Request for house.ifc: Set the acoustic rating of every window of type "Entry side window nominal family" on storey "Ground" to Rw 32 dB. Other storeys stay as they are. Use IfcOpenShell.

First a look at what the model holds.

```python
import ifcopenshell
import ifcopenshell.util.element

model = ifcopenshell.open("house.ifc")
print(model.schema)
storey = next(s for s in model.by_type("IfcBuildingStorey") if s.Name == "Ground")
windows = [e for e in ifcopenshell.util.element.get_decomposition(storey) if e.is_a("IfcWindow")]
seen = {}
for e in windows:
    element_type = ifcopenshell.util.element.get_type(e)
    key = (element_type.Name if element_type != e and element_type else None, ifcopenshell.util.element.get_pset(e, "Pset_WindowCommon", "AcousticRating"))
    seen[key] = seen.get(key, 0) + 1
for (name, value), count in sorted(seen.items(), key=str):
    print(count, "x", name, "|", value)
```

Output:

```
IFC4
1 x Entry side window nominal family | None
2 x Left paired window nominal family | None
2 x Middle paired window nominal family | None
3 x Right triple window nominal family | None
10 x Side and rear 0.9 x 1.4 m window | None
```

```python
import ifcopenshell
import ifcopenshell.api.pset
import ifcopenshell.util.element

model = ifcopenshell.open("house.ifc")

storey = next(s for s in model.by_type("IfcBuildingStorey") if s.Name == "Ground")
windows = [e for e in ifcopenshell.util.element.get_decomposition(storey) if e.is_a("IfcWindow")]

count = 0
for e in windows:
    element_type = ifcopenshell.util.element.get_type(e)
    if element_type in (None, e) or element_type.Name != "Entry side window nominal family":
        continue
    # add_pset returns the element's existing set when there is one.
    pset = ifcopenshell.api.pset.add_pset(model, product=e, name="Pset_WindowCommon")
    ifcopenshell.api.pset.edit_pset(model, pset=pset, properties={"AcousticRating": "Rw 32 dB"})
    count += 1

print(count, "windows updated")

model.write("house_rev.ifc")
```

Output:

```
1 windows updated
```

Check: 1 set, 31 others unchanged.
